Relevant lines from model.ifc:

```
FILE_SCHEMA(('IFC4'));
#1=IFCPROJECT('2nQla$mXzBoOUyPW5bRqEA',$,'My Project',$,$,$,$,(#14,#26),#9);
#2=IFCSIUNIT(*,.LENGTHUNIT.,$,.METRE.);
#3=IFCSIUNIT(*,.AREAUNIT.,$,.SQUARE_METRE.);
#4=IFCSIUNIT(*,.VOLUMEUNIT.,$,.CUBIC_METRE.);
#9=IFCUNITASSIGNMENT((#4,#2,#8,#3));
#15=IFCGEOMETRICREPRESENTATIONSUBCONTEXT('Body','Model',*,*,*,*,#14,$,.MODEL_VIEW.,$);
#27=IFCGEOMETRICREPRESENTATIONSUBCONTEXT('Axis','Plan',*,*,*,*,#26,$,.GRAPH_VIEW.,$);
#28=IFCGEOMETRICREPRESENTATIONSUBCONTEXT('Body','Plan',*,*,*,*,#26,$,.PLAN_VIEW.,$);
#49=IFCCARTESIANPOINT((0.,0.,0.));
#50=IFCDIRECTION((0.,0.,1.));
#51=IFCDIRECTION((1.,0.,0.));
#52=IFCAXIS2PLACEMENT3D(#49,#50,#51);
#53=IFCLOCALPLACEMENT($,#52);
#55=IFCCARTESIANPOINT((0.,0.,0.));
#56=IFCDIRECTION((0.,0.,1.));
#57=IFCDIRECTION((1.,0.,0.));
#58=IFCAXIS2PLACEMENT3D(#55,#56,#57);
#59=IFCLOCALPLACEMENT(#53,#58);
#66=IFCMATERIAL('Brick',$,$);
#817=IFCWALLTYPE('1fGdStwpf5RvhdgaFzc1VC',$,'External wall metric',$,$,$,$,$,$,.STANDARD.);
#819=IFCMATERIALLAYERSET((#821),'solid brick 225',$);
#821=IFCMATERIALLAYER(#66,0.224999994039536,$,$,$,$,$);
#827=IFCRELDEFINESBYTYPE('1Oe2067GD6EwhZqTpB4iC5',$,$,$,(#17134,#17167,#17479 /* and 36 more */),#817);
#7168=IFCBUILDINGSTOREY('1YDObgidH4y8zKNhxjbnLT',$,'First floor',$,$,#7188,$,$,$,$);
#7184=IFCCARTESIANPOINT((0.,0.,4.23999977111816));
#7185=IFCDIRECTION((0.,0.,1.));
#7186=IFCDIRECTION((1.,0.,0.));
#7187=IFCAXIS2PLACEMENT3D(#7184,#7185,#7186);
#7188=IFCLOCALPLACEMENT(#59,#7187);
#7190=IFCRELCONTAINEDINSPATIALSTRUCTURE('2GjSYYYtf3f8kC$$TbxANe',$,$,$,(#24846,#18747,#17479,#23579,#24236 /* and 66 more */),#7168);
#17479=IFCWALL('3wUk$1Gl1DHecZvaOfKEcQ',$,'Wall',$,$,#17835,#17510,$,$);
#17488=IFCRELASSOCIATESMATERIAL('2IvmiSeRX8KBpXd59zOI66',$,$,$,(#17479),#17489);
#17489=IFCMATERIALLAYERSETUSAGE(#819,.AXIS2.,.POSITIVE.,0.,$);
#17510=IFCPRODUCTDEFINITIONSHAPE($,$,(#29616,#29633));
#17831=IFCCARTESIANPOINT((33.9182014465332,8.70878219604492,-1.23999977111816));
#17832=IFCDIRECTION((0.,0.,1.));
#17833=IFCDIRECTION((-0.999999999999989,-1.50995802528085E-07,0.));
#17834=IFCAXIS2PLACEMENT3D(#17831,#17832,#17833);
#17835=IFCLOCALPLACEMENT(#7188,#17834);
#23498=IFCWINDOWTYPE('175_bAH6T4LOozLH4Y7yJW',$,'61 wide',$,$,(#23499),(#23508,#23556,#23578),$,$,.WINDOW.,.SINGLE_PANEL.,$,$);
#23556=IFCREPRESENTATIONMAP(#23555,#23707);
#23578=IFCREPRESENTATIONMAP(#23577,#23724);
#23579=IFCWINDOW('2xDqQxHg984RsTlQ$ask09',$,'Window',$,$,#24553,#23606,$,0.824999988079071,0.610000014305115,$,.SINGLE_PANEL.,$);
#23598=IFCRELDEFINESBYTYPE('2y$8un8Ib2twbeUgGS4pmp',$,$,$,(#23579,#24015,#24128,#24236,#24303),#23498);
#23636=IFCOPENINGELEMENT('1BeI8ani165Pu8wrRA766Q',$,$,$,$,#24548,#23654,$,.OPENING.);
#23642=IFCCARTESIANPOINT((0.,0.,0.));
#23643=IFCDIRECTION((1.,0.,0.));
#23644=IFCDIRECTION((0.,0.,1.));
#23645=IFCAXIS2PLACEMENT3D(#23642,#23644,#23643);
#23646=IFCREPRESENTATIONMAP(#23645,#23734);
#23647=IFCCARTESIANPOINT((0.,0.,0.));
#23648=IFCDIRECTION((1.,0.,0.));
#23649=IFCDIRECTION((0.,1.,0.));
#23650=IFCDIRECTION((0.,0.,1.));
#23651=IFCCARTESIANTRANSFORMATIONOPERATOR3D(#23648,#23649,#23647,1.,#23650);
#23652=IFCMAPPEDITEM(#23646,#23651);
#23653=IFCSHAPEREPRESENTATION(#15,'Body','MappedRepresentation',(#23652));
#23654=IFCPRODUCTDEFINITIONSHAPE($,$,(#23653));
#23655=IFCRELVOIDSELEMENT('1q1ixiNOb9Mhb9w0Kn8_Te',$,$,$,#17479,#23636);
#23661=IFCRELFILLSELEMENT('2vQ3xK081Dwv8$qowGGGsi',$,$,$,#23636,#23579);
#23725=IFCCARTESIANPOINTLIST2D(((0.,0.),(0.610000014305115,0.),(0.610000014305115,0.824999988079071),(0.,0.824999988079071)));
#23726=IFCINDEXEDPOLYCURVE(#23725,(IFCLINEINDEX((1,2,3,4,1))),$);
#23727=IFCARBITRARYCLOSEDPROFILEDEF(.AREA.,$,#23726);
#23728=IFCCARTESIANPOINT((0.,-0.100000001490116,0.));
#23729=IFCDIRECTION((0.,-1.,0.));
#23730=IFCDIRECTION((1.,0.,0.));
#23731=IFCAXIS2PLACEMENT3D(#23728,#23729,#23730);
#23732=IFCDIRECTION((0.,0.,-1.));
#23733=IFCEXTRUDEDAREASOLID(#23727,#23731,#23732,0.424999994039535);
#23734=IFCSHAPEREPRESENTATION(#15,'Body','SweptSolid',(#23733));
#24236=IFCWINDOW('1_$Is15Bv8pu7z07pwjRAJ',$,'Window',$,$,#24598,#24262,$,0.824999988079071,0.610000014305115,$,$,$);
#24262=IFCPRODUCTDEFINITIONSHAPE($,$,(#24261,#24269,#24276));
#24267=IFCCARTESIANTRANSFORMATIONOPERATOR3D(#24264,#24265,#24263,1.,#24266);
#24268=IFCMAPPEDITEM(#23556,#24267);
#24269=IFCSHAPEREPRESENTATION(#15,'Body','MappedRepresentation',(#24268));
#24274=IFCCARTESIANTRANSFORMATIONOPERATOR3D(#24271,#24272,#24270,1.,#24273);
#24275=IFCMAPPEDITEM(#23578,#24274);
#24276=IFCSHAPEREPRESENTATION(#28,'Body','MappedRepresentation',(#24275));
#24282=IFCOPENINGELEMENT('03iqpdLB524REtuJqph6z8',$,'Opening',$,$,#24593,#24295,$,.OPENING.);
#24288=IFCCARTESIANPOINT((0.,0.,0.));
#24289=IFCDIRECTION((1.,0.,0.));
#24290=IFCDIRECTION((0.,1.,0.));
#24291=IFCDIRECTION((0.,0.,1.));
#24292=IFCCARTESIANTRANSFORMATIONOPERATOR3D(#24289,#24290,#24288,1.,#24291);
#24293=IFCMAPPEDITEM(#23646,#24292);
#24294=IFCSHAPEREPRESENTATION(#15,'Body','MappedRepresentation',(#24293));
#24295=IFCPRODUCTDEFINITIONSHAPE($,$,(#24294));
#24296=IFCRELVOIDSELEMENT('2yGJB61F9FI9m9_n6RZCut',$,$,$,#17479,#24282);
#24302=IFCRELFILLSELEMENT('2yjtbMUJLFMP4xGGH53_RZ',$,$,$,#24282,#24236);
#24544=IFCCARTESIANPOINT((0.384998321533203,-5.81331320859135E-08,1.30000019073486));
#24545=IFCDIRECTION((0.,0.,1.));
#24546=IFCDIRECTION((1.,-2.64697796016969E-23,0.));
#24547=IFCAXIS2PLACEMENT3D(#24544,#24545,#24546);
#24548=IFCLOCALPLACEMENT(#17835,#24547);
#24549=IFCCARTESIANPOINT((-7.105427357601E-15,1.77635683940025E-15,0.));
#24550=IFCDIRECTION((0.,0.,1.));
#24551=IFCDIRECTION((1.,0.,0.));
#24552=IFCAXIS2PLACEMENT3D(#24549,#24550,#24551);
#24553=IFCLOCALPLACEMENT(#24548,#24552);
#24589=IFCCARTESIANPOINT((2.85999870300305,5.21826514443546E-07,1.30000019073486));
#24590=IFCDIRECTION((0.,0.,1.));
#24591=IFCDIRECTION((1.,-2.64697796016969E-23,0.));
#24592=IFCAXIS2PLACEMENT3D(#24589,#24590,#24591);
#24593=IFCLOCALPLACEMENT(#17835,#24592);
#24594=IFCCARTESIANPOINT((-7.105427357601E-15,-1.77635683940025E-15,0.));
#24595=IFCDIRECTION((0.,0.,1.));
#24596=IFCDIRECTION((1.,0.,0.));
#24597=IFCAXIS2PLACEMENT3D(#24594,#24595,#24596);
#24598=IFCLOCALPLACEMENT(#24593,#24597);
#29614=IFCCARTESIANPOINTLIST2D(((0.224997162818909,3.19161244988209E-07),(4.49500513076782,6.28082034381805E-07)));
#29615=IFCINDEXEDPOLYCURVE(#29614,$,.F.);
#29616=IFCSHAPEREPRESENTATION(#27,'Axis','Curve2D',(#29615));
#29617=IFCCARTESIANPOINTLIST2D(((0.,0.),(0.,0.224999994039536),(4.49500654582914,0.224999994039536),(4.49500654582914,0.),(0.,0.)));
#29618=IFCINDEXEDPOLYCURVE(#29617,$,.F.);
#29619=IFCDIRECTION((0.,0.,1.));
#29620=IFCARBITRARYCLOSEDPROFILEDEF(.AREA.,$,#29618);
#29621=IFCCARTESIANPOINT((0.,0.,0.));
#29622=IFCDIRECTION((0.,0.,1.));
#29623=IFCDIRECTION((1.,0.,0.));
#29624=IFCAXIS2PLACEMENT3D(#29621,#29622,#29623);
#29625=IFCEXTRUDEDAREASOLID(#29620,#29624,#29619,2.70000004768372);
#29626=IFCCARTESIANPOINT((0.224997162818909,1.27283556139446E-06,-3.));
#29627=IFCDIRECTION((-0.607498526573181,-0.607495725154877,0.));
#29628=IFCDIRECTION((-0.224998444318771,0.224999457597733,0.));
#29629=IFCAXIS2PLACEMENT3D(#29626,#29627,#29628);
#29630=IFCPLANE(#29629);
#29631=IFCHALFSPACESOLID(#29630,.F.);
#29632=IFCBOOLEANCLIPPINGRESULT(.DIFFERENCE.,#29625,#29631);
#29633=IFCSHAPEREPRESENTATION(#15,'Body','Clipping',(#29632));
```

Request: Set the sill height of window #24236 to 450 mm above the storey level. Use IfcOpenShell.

```python
import numpy as np
import ifcopenshell
import ifcopenshell.api.geometry
import ifcopenshell.geom
import ifcopenshell.util.element
import ifcopenshell.util.placement
import ifcopenshell.util.shape
import ifcopenshell.util.unit

model = ifcopenshell.open("model.ifc")
unit_scale = ifcopenshell.util.unit.calculate_unit_scale(model)

window = model.by_guid("1_$Is15Bv8pu7z07pwjRAJ")
opening = window.FillsVoids[0].RelatingOpeningElement
storey = ifcopenshell.util.element.get_container(window, ifc_class="IfcBuildingStorey")
level = ifcopenshell.util.placement.get_local_placement(storey.ObjectPlacement)[2, 3]

# The opening's origin need not be at the sill, so measure its lowest point.
shape = ifcopenshell.geom.create_shape(ifcopenshell.geom.settings(), opening)
bottom = ifcopenshell.util.shape.get_shape_bottom_elevation(shape, shape.geometry) / unit_scale
dz = level + 0.45 / unit_scale - bottom

shift = np.array([0.0, 0.0, dz])
# The window is placed relative to its opening, so it follows when the opening moves.
matrix = ifcopenshell.util.placement.get_local_placement(opening.ObjectPlacement)
matrix[:3, 3] += shift
ifcopenshell.api.geometry.edit_object_placement(
    model, product=opening, matrix=matrix, is_si=False, should_transform_children=True
)

print(f"moved by {dz * unit_scale:+.3f} m")

model.write("model_edited.ifc")
```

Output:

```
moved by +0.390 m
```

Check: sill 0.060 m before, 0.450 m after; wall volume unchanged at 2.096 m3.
